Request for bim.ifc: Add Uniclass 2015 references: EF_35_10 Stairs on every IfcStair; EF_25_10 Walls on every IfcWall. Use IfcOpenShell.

First a look at what the model holds.

```python
import ifcopenshell

model = ifcopenshell.open("bim.ifc")
print(model.schema)
print("classifications:", [c.Name for c in model.by_type("IfcClassification")])
for ifc_class in ("IfcDoor", "IfcRoof", "IfcStair", "IfcWall", "IfcWindow"):
    print(ifc_class, len(model.by_type(ifc_class)))
```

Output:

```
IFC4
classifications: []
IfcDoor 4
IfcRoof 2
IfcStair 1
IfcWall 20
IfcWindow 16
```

```python
import ifcopenshell
import ifcopenshell.api.classification

model = ifcopenshell.open("bim.ifc")

system = ifcopenshell.api.classification.add_classification(model, classification="Uniclass 2015")

codes = {
    "IfcStair": ("EF_35_10", "Stairs"),
    "IfcWall": ("EF_25_10", "Walls"),
}
for ifc_class, (code, name) in codes.items():
    products = model.by_type(ifc_class)
    ifcopenshell.api.classification.add_reference(
        model, products=products, classification=system, identification=code, name=name
    )
    print(code, len(products))

model.write("bim_rev.ifc")
```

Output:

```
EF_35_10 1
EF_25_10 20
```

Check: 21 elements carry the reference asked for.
